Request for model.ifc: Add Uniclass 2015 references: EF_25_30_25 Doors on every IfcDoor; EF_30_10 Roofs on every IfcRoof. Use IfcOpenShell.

First a look at what the model holds.

```python
import ifcopenshell

model = ifcopenshell.open("model.ifc")
print(model.schema)
print("classifications:", [c.Name for c in model.by_type("IfcClassification")])
for ifc_class in ("IfcDoor", "IfcRoof", "IfcStair", "IfcWall", "IfcWindow"):
    print(ifc_class, len(model.by_type(ifc_class)))
```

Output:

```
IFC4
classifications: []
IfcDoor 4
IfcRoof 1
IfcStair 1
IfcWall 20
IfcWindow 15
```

```python
import ifcopenshell
import ifcopenshell.api.classification

model = ifcopenshell.open("model.ifc")

system = ifcopenshell.api.classification.add_classification(model, classification="Uniclass 2015")

codes = {
    "IfcDoor": ("EF_25_30_25", "Doors"),
    "IfcRoof": ("EF_30_10", "Roofs"),
}
for ifc_class, (code, name) in codes.items():
    products = model.by_type(ifc_class)
    ifcopenshell.api.classification.add_reference(
        model, products=products, classification=system, identification=code, name=name
    )
    print(code, len(products))

model.write("model_rev.ifc")
```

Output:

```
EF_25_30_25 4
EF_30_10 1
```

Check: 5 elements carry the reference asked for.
